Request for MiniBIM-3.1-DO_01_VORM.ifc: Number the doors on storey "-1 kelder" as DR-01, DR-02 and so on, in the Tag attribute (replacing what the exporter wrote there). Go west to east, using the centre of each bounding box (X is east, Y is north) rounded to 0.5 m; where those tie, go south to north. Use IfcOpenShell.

First a look at what the model holds.

```python
import ifcopenshell
import ifcopenshell.util.element
import ifcopenshell.util.placement

model = ifcopenshell.open("MiniBIM-3.1-DO_01_VORM.ifc")
print(model.schema)
storey = next(s for s in model.by_type("IfcBuildingStorey") if s.Name == "-1 kelder")
doors = [e for e in ifcopenshell.util.element.get_decomposition(storey) if e.is_a("IfcDoor")]
for e in sorted(doors, key=lambda e: e.id()):
    origin = ifcopenshell.util.placement.get_local_placement(e.ObjectPlacement)[:3, 3]
    print(e.id(), e.Tag, e.Name, origin.round(2) + 0.0, sep=" | ")
```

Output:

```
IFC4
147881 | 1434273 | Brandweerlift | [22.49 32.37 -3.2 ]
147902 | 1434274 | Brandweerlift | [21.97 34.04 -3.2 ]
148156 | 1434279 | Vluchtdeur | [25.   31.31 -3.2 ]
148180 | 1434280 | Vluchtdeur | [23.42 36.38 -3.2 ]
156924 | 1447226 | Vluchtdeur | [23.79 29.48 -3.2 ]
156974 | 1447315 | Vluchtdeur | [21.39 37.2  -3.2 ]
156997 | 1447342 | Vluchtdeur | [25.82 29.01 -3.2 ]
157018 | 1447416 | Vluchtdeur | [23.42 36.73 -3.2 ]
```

```python
import ifcopenshell
import ifcopenshell.geom
import ifcopenshell.util.element
import ifcopenshell.util.shape

model = ifcopenshell.open("MiniBIM-3.1-DO_01_VORM.ifc")
settings = ifcopenshell.geom.settings()
settings.set("use-world-coords", True)


def centre(element):
    shape = ifcopenshell.geom.create_shape(settings, element)
    return ifcopenshell.util.shape.get_bbox_centroid(shape.geometry)


storey = next(s for s in model.by_type("IfcBuildingStorey") if s.Name == "-1 kelder")
doors = [e for e in ifcopenshell.util.element.get_decomposition(storey) if e.is_a("IfcDoor")]

# Insertion points can sit at a corner or the storey origin, so sort by the geometry (in metres).
centres = {e: centre(e) for e in doors}
doors.sort(key=lambda e: (round(centres[e][0] / 0.5), centres[e][1]))

for i, e in enumerate(doors, start=1):
    number = f"DR-{i:02d}"
    e.Tag = number
    print(e.id(), number)

model.write("MiniBIM-3.1-DO_01_VORM_v2.ifc")
```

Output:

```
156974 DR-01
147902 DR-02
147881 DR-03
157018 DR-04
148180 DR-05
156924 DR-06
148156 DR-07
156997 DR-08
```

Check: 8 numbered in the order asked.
